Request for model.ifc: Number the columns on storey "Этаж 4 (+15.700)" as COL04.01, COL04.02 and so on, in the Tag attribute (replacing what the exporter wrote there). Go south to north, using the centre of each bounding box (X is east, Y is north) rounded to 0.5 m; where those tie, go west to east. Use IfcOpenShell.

First a look at what the model holds.

```python
import ifcopenshell
import ifcopenshell.util.element
import ifcopenshell.util.placement

model = ifcopenshell.open("model.ifc")
print(model.schema)
storey = next(s for s in model.by_type("IfcBuildingStorey") if s.Name == "Этаж 4 (+15.700)")
columns = [e for e in ifcopenshell.util.element.get_decomposition(storey) if e.is_a("IfcColumn")]
for e in sorted(columns, key=lambda e: e.id()):
    origin = ifcopenshell.util.placement.get_local_placement(e.ObjectPlacement)[:3, 3]
    print(e.id(), e.Tag, e.Name, origin.round(2) + 0.0, sep=" | ")
```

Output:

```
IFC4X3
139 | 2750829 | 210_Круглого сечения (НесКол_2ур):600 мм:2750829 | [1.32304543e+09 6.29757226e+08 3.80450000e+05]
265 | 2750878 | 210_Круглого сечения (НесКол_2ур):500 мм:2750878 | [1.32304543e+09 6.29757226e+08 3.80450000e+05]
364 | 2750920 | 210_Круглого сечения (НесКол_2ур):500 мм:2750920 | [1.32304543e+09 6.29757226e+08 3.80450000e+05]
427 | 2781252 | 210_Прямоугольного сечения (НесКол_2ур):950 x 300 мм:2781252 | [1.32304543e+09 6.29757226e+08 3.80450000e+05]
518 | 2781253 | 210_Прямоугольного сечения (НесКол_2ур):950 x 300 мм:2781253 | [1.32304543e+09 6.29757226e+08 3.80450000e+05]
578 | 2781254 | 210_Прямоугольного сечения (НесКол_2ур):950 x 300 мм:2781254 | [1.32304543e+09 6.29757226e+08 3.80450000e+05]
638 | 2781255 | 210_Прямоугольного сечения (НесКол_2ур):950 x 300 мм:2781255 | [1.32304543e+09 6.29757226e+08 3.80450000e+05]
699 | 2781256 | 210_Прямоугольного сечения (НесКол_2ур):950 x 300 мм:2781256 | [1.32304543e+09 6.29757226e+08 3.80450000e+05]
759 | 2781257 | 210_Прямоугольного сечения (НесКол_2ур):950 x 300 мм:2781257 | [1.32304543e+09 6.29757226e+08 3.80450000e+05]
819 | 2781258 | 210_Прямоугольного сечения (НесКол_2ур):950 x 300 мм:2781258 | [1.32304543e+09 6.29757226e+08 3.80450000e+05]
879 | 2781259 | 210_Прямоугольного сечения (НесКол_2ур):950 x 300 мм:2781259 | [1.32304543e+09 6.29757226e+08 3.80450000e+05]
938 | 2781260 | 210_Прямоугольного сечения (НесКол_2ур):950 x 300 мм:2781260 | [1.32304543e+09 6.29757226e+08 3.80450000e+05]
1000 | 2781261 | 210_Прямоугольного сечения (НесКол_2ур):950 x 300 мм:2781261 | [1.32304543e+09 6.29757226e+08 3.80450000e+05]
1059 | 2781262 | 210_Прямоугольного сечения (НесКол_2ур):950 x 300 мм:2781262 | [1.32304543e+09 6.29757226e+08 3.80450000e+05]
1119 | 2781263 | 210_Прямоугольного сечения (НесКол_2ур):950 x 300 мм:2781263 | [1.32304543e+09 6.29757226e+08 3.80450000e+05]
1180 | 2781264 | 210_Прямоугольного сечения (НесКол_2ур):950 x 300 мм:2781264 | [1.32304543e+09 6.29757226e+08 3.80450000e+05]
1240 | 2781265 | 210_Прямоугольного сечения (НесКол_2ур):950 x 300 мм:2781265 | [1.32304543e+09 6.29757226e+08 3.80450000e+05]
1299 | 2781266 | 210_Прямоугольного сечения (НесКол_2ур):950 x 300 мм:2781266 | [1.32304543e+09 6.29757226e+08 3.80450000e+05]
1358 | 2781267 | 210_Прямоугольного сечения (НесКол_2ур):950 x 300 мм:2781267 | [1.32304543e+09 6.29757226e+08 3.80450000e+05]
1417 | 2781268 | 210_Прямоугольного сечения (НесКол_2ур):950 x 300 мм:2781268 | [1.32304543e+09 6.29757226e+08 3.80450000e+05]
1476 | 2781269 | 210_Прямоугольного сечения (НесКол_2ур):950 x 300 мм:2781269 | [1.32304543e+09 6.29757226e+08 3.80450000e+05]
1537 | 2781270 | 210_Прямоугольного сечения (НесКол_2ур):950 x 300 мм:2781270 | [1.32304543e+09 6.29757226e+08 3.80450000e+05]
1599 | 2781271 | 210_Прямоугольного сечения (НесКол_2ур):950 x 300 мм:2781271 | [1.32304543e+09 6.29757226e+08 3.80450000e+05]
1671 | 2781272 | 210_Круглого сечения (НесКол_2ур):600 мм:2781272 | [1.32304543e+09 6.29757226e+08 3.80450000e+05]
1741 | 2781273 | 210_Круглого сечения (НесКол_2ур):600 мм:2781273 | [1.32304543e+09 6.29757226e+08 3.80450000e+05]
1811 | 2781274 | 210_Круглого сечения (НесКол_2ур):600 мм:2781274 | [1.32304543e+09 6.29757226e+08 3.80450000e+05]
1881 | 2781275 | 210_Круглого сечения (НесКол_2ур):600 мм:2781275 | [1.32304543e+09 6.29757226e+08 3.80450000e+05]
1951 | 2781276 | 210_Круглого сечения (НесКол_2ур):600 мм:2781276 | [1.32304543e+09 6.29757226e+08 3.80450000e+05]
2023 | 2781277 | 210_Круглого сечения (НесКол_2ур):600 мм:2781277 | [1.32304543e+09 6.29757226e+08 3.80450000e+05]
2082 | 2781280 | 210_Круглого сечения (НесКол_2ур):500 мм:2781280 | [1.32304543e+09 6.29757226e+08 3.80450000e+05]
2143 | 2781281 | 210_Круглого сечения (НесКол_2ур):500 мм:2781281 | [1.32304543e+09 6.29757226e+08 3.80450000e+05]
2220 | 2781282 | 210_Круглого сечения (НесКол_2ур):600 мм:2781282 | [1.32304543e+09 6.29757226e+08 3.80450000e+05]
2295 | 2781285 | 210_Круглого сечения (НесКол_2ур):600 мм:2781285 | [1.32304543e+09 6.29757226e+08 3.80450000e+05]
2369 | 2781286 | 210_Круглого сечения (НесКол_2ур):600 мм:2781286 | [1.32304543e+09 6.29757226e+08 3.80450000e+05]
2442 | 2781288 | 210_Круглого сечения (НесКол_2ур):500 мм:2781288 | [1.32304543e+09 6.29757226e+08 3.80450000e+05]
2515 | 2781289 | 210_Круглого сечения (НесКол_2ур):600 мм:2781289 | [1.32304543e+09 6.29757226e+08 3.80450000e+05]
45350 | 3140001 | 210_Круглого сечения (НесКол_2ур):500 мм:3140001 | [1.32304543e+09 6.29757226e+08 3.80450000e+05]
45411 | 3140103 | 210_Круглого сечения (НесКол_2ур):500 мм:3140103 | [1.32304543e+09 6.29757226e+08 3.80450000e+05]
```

```python
import ifcopenshell
import ifcopenshell.geom
import ifcopenshell.util.element
import ifcopenshell.util.shape

model = ifcopenshell.open("model.ifc")
settings = ifcopenshell.geom.settings()
settings.set("use-world-coords", True)


def centre(element):
    shape = ifcopenshell.geom.create_shape(settings, element)
    return ifcopenshell.util.shape.get_bbox_centroid(shape.geometry)


storey = next(s for s in model.by_type("IfcBuildingStorey") if s.Name == "Этаж 4 (+15.700)")
columns = [e for e in ifcopenshell.util.element.get_decomposition(storey) if e.is_a("IfcColumn")]

# Insertion points can sit at a corner or the storey origin, so sort by the geometry (in metres).
centres = {e: centre(e) for e in columns}
columns.sort(key=lambda e: (round(centres[e][1] / 0.5), centres[e][0]))

for i, e in enumerate(columns, start=1):
    number = f"COL04.{i:02d}"
    e.Tag = number
    print(e.id(), number)

model.write("model_updated.ifc")
```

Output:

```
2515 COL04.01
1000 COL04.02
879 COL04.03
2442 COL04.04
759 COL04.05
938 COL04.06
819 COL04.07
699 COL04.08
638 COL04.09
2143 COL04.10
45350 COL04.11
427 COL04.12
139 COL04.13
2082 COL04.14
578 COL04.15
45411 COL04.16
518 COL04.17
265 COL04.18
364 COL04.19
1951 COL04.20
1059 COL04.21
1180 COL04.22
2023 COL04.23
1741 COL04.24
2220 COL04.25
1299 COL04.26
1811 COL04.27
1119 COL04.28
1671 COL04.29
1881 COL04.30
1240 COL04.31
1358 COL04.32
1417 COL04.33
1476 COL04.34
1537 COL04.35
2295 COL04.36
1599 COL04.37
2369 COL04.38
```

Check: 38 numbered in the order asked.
